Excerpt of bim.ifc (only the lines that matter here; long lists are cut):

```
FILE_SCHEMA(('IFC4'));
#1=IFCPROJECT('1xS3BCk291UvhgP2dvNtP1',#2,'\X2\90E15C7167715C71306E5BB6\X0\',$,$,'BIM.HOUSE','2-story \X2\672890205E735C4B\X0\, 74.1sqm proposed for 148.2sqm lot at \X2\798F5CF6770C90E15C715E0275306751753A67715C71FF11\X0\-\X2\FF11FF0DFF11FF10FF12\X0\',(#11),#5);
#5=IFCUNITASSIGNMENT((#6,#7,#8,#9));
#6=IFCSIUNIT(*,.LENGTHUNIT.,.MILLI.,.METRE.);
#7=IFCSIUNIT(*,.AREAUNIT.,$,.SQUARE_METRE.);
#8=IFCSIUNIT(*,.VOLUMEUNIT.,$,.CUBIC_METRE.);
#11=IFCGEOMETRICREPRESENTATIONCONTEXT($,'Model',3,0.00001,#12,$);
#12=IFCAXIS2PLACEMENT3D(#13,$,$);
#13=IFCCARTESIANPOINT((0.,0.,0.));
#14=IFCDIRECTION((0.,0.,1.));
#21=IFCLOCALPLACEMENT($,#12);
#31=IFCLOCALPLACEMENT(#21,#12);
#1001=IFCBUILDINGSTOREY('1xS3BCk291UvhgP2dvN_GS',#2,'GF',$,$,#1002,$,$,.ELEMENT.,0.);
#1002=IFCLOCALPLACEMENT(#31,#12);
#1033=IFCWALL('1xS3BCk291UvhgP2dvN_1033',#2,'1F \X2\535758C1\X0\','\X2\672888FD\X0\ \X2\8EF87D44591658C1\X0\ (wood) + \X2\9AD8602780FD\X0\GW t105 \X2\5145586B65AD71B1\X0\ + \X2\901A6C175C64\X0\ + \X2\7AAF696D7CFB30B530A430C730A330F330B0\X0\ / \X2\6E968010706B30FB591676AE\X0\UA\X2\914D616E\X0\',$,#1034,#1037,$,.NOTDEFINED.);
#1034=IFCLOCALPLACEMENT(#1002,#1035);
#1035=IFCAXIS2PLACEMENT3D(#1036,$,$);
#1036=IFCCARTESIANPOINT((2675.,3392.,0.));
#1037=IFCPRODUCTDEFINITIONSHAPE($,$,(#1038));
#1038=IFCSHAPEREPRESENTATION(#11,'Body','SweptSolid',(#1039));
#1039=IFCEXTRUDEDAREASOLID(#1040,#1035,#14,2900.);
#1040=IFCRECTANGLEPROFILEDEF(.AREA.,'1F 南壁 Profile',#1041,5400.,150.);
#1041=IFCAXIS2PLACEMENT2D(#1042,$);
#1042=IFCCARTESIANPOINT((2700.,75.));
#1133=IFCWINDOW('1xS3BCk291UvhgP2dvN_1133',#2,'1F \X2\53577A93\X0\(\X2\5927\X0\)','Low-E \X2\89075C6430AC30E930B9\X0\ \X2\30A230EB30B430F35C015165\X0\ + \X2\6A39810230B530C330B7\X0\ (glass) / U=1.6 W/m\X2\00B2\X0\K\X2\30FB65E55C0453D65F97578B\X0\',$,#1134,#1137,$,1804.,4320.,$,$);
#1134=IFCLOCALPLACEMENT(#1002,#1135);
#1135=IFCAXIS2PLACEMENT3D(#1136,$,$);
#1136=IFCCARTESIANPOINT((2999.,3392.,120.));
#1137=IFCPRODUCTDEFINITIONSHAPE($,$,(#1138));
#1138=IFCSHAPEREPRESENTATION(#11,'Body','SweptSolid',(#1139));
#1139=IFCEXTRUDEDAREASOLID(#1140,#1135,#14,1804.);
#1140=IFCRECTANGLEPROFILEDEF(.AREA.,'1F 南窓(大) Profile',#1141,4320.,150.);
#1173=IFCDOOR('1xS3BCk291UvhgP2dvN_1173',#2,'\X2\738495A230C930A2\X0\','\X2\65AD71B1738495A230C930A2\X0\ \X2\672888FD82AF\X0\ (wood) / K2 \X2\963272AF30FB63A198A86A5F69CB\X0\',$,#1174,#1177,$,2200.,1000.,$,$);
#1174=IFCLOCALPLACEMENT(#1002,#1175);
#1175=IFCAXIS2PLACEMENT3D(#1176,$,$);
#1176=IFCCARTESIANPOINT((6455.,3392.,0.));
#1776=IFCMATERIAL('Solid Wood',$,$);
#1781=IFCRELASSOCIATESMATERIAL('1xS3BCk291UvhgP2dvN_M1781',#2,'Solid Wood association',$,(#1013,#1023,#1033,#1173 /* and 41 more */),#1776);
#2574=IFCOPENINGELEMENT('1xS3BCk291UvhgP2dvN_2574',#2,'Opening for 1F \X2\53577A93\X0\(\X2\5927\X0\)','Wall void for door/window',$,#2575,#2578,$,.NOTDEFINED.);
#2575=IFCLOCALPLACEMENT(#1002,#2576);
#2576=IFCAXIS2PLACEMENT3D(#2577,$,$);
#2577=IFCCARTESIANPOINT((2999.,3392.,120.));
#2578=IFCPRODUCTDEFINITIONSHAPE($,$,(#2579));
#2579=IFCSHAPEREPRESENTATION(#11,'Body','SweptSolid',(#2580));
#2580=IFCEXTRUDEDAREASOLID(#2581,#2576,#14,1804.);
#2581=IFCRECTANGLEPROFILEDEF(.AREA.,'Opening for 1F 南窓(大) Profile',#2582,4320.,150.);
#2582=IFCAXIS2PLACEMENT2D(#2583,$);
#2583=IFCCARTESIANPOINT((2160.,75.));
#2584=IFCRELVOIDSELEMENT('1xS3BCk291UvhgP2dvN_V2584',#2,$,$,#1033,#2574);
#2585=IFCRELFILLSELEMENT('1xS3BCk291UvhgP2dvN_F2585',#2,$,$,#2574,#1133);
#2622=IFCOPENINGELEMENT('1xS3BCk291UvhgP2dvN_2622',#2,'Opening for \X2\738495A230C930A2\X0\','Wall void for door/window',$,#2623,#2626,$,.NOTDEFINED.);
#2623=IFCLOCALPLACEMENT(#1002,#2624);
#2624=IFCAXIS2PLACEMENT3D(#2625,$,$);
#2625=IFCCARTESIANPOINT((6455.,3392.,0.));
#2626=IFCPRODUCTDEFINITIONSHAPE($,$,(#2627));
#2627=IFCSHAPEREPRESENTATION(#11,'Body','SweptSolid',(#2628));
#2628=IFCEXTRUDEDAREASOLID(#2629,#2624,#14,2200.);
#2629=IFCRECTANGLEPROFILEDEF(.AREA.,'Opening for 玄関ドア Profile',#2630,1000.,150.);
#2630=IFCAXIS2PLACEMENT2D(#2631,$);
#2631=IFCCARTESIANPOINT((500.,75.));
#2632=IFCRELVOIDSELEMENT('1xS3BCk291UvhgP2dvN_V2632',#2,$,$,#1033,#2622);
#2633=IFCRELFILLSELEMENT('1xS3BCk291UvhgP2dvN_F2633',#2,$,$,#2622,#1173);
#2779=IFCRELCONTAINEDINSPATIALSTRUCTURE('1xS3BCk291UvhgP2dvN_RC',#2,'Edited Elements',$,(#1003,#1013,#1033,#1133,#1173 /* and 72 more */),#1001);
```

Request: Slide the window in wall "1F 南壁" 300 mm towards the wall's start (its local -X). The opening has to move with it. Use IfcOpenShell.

```python
import ifcopenshell
import ifcopenshell.api.geometry
import ifcopenshell.util.placement

model = ifcopenshell.open("bim.ifc")

window = model.by_guid("1xS3BCk291UvhgP2dvN_1133")
opening = window.FillsVoids[0].RelatingOpeningElement
wall = opening.VoidsElements[0].RelatingBuildingElement

wall_matrix = ifcopenshell.util.placement.get_local_placement(wall.ObjectPlacement)
shift = wall_matrix[:3, 0] * -300.0
before = ifcopenshell.util.placement.get_local_placement(window.ObjectPlacement)[:3, 3].copy()

# The window is not placed relative to its opening, so move both.
for product in (opening, window):
    matrix = ifcopenshell.util.placement.get_local_placement(product.ObjectPlacement)
    matrix[:3, 3] += shift
    ifcopenshell.api.geometry.edit_object_placement(model, product=product, matrix=matrix, is_si=False)

after = ifcopenshell.util.placement.get_local_placement(window.ObjectPlacement)[:3, 3]
print("window moved by", (after - before).round(3) + 0.0)

model.write("bim_v2.ifc")
```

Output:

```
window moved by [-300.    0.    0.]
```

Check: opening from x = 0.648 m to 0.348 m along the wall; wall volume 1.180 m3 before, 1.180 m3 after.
